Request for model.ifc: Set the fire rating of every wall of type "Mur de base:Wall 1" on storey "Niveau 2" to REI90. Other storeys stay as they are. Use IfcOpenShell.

First a look at what the model holds.

```python
import ifcopenshell
import ifcopenshell.util.element

model = ifcopenshell.open("model.ifc")
print(model.schema)
storey = next(s for s in model.by_type("IfcBuildingStorey") if s.Name == "Niveau 2")
walls = [e for e in ifcopenshell.util.element.get_decomposition(storey) if e.is_a("IfcWall")]
seen = {}
for e in walls:
    element_type = ifcopenshell.util.element.get_type(e)
    key = (element_type.Name if element_type != e and element_type else None, ifcopenshell.util.element.get_pset(e, "Pset_WallCommon", "FireRating"))
    seen[key] = seen.get(key, 0) + 1
for (name, value), count in sorted(seen.items(), key=str):
    print(count, "x", name, "|", value)
```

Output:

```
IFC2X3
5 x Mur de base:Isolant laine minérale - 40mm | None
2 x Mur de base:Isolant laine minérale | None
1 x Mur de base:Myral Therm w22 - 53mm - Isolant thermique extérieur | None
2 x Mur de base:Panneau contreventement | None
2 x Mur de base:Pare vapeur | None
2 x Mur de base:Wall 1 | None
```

```python
import ifcopenshell
import ifcopenshell.api.pset
import ifcopenshell.util.element

model = ifcopenshell.open("model.ifc")

storey = next(s for s in model.by_type("IfcBuildingStorey") if s.Name == "Niveau 2")
walls = [e for e in ifcopenshell.util.element.get_decomposition(storey) if e.is_a("IfcWall")]

count = 0
for e in walls:
    element_type = ifcopenshell.util.element.get_type(e)
    if element_type in (None, e) or element_type.Name != "Mur de base:Wall 1":
        continue
    # add_pset returns the element's existing set when there is one.
    pset = ifcopenshell.api.pset.add_pset(model, product=e, name="Pset_WallCommon")
    ifcopenshell.api.pset.edit_pset(model, pset=pset, properties={"FireRating": "REI90"})
    count += 1

print(count, "walls updated")

model.write("model_updated.ifc")
```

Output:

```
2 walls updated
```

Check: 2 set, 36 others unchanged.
